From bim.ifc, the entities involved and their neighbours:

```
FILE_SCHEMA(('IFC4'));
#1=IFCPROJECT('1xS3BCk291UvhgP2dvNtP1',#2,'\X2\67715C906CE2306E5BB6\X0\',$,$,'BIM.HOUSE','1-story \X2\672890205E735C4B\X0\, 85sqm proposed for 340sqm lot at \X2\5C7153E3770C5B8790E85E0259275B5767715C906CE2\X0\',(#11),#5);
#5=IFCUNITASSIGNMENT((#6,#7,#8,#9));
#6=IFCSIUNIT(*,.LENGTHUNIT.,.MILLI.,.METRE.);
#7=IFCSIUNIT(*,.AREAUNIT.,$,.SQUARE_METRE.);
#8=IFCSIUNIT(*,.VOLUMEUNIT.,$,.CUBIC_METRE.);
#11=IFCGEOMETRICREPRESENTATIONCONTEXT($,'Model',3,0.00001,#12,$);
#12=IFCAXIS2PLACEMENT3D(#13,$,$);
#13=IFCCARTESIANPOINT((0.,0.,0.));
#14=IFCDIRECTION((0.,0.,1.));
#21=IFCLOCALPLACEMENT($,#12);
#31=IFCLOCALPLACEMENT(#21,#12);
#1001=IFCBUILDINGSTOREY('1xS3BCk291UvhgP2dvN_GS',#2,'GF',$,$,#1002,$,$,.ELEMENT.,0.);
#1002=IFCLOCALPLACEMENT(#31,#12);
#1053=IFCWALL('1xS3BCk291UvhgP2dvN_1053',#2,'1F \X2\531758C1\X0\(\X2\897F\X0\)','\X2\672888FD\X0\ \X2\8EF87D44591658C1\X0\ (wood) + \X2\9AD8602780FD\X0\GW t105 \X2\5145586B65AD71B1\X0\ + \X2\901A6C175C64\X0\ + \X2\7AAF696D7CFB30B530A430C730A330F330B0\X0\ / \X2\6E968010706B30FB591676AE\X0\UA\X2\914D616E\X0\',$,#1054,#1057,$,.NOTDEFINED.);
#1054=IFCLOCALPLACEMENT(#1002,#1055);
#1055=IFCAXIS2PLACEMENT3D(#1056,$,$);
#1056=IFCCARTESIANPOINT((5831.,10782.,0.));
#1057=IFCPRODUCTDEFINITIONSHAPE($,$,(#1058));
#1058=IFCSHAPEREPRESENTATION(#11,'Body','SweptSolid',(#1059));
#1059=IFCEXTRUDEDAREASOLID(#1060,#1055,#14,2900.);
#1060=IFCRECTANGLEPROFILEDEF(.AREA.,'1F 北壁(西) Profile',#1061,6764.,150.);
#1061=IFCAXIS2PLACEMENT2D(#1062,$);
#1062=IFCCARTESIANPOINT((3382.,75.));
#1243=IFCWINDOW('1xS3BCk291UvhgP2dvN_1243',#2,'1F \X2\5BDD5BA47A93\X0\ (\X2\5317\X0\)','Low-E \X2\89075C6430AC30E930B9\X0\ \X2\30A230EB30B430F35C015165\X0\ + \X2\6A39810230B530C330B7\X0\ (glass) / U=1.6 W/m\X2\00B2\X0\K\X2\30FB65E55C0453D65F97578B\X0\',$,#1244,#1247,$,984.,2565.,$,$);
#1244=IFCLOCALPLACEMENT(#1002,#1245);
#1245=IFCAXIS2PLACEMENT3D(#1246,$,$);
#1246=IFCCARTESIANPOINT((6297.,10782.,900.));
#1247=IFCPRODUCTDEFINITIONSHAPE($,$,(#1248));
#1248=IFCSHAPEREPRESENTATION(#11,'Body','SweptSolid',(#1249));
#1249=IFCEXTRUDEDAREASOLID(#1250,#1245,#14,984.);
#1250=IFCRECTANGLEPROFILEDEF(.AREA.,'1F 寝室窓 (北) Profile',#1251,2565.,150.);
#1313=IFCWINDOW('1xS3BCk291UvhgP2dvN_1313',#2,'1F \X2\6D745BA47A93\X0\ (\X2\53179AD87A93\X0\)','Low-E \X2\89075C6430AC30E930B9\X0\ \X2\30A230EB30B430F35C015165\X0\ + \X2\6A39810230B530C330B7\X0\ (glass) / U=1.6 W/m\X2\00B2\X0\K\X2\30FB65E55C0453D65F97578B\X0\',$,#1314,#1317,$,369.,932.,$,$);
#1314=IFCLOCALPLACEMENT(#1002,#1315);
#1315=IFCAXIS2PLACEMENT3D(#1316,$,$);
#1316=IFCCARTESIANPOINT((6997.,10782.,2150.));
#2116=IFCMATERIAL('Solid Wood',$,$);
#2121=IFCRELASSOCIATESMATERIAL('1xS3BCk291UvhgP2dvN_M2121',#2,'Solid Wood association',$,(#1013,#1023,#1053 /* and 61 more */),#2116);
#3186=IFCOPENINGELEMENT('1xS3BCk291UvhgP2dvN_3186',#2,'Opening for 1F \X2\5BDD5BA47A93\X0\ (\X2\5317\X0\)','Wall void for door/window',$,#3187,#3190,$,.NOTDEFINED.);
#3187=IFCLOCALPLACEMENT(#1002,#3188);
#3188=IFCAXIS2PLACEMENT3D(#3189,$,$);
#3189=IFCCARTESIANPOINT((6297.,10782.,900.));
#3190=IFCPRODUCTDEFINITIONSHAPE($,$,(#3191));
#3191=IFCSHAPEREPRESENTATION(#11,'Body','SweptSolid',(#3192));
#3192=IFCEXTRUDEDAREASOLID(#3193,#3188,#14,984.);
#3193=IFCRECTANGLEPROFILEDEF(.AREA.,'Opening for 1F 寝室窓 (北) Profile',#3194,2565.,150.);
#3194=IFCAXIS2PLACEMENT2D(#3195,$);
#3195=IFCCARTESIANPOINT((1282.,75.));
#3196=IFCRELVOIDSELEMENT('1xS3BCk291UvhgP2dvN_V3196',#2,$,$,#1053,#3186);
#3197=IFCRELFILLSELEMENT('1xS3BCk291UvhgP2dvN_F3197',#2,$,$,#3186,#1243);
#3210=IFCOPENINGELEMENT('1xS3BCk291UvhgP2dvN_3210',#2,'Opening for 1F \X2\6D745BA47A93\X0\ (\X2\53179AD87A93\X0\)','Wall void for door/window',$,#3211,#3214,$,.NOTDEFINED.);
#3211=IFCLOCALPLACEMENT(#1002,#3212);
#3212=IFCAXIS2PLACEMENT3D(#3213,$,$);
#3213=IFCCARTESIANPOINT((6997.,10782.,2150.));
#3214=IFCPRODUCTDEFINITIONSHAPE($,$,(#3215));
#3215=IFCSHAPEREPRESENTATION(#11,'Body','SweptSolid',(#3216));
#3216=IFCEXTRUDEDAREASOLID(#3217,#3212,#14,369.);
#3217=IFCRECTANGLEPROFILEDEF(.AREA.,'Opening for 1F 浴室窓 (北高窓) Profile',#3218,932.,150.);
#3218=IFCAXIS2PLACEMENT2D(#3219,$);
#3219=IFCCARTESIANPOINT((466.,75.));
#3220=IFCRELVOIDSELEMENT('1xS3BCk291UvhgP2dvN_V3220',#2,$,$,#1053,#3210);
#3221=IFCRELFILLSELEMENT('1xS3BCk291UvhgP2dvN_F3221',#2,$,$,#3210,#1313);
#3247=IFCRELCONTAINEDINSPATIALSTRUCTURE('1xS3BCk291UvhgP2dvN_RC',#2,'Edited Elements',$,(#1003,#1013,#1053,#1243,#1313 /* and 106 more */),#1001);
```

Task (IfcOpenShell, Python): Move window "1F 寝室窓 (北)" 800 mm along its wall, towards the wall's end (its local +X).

```python
import ifcopenshell
import ifcopenshell.api.geometry
import ifcopenshell.util.placement

model = ifcopenshell.open("bim.ifc")

window = model.by_guid("1xS3BCk291UvhgP2dvN_1243")
opening = window.FillsVoids[0].RelatingOpeningElement
wall = opening.VoidsElements[0].RelatingBuildingElement

wall_matrix = ifcopenshell.util.placement.get_local_placement(wall.ObjectPlacement)
shift = wall_matrix[:3, 0] * 800.0
before = ifcopenshell.util.placement.get_local_placement(window.ObjectPlacement)[:3, 3].copy()

# The window is not placed relative to its opening, so move both.
for product in (opening, window):
    matrix = ifcopenshell.util.placement.get_local_placement(product.ObjectPlacement)
    matrix[:3, 3] += shift
    ifcopenshell.api.geometry.edit_object_placement(model, product=product, matrix=matrix, is_si=False)

after = ifcopenshell.util.placement.get_local_placement(window.ObjectPlacement)[:3, 3]
print("window moved by", (after - before).round(3) + 0.0)

model.write("bim_edited.ifc")
```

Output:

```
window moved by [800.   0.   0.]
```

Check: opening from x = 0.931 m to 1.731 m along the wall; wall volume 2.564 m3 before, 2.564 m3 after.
